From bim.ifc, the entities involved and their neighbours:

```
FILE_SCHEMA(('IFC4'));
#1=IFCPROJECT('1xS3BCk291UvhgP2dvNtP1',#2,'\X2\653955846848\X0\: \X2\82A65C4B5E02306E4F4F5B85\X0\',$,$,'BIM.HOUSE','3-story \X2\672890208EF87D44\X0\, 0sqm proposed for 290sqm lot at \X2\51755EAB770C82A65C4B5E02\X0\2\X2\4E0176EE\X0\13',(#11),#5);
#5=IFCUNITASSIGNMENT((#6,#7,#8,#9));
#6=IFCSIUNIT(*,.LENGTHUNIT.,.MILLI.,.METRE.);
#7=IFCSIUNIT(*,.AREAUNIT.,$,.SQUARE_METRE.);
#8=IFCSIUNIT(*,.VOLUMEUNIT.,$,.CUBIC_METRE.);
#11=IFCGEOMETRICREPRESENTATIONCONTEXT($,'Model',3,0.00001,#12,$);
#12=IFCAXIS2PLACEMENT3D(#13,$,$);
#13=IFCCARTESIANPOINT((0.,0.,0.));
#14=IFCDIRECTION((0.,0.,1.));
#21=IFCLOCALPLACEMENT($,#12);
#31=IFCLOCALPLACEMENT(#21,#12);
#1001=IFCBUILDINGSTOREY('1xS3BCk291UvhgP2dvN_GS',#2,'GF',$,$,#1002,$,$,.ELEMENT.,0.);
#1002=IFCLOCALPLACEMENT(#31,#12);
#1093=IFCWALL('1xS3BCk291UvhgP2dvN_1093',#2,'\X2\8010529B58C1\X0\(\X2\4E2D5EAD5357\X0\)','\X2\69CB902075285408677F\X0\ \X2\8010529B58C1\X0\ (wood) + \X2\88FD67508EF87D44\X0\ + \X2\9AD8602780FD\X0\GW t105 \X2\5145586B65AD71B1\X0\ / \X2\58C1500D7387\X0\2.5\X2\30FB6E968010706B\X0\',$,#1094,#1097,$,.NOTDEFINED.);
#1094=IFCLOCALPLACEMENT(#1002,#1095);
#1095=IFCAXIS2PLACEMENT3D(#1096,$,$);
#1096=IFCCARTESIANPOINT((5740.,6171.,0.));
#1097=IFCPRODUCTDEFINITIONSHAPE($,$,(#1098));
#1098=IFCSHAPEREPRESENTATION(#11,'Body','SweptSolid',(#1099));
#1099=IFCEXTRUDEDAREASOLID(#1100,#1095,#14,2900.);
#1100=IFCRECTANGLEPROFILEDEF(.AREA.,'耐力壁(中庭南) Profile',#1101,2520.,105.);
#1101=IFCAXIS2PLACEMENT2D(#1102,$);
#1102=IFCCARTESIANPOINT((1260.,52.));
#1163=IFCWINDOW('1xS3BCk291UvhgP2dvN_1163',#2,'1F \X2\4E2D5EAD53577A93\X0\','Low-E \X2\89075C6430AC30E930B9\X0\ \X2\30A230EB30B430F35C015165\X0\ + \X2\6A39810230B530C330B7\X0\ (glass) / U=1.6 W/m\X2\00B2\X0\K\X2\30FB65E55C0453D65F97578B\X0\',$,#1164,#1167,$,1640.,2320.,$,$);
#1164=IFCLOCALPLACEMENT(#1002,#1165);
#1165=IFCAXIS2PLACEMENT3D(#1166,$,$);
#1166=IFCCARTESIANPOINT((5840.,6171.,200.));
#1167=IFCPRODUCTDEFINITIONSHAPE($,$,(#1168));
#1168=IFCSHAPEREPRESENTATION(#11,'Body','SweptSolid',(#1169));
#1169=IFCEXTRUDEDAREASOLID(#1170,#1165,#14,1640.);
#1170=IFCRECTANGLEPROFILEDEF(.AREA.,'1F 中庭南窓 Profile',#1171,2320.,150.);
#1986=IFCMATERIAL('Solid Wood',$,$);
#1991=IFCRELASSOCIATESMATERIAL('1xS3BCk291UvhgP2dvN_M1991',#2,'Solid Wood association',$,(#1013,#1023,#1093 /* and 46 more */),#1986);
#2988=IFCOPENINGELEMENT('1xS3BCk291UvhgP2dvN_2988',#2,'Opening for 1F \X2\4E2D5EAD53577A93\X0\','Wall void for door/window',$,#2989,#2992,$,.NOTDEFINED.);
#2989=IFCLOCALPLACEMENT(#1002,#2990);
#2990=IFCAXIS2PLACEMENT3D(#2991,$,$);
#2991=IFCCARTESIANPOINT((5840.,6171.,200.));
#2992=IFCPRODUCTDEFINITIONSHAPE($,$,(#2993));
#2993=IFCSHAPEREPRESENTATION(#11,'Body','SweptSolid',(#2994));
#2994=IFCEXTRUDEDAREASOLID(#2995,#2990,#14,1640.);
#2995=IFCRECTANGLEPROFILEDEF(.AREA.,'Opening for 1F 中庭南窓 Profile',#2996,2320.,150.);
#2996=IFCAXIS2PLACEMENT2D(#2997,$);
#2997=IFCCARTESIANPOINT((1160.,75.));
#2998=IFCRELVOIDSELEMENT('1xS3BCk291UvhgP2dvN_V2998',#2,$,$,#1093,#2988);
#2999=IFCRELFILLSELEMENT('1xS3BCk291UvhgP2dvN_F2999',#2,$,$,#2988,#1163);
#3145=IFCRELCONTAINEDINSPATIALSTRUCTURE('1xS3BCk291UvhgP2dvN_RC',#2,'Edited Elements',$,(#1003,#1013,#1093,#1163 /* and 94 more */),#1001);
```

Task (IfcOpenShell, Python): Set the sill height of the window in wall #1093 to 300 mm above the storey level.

```python
import numpy as np
import ifcopenshell
import ifcopenshell.api.geometry
import ifcopenshell.geom
import ifcopenshell.util.element
import ifcopenshell.util.placement
import ifcopenshell.util.shape
import ifcopenshell.util.unit

model = ifcopenshell.open("bim.ifc")
unit_scale = ifcopenshell.util.unit.calculate_unit_scale(model)

window = model.by_guid("1xS3BCk291UvhgP2dvN_1163")
opening = window.FillsVoids[0].RelatingOpeningElement
storey = ifcopenshell.util.element.get_container(window, ifc_class="IfcBuildingStorey")
level = ifcopenshell.util.placement.get_local_placement(storey.ObjectPlacement)[2, 3]

# The opening's origin need not be at the sill, so measure its lowest point.
shape = ifcopenshell.geom.create_shape(ifcopenshell.geom.settings(), opening)
bottom = ifcopenshell.util.shape.get_shape_bottom_elevation(shape, shape.geometry) / unit_scale
dz = level + 300.0 - bottom

shift = np.array([0.0, 0.0, dz])
# The window is not placed relative to its opening, so move both.
for product in (opening, window):
    matrix = ifcopenshell.util.placement.get_local_placement(product.ObjectPlacement)
    matrix[:3, 3] += shift
    ifcopenshell.api.geometry.edit_object_placement(model, product=product, matrix=matrix, is_si=False)

print(f"moved by {dz * unit_scale:+.3f} m")

model.write("bim-out.ifc")
```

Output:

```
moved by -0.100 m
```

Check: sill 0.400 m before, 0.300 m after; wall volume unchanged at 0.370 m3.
